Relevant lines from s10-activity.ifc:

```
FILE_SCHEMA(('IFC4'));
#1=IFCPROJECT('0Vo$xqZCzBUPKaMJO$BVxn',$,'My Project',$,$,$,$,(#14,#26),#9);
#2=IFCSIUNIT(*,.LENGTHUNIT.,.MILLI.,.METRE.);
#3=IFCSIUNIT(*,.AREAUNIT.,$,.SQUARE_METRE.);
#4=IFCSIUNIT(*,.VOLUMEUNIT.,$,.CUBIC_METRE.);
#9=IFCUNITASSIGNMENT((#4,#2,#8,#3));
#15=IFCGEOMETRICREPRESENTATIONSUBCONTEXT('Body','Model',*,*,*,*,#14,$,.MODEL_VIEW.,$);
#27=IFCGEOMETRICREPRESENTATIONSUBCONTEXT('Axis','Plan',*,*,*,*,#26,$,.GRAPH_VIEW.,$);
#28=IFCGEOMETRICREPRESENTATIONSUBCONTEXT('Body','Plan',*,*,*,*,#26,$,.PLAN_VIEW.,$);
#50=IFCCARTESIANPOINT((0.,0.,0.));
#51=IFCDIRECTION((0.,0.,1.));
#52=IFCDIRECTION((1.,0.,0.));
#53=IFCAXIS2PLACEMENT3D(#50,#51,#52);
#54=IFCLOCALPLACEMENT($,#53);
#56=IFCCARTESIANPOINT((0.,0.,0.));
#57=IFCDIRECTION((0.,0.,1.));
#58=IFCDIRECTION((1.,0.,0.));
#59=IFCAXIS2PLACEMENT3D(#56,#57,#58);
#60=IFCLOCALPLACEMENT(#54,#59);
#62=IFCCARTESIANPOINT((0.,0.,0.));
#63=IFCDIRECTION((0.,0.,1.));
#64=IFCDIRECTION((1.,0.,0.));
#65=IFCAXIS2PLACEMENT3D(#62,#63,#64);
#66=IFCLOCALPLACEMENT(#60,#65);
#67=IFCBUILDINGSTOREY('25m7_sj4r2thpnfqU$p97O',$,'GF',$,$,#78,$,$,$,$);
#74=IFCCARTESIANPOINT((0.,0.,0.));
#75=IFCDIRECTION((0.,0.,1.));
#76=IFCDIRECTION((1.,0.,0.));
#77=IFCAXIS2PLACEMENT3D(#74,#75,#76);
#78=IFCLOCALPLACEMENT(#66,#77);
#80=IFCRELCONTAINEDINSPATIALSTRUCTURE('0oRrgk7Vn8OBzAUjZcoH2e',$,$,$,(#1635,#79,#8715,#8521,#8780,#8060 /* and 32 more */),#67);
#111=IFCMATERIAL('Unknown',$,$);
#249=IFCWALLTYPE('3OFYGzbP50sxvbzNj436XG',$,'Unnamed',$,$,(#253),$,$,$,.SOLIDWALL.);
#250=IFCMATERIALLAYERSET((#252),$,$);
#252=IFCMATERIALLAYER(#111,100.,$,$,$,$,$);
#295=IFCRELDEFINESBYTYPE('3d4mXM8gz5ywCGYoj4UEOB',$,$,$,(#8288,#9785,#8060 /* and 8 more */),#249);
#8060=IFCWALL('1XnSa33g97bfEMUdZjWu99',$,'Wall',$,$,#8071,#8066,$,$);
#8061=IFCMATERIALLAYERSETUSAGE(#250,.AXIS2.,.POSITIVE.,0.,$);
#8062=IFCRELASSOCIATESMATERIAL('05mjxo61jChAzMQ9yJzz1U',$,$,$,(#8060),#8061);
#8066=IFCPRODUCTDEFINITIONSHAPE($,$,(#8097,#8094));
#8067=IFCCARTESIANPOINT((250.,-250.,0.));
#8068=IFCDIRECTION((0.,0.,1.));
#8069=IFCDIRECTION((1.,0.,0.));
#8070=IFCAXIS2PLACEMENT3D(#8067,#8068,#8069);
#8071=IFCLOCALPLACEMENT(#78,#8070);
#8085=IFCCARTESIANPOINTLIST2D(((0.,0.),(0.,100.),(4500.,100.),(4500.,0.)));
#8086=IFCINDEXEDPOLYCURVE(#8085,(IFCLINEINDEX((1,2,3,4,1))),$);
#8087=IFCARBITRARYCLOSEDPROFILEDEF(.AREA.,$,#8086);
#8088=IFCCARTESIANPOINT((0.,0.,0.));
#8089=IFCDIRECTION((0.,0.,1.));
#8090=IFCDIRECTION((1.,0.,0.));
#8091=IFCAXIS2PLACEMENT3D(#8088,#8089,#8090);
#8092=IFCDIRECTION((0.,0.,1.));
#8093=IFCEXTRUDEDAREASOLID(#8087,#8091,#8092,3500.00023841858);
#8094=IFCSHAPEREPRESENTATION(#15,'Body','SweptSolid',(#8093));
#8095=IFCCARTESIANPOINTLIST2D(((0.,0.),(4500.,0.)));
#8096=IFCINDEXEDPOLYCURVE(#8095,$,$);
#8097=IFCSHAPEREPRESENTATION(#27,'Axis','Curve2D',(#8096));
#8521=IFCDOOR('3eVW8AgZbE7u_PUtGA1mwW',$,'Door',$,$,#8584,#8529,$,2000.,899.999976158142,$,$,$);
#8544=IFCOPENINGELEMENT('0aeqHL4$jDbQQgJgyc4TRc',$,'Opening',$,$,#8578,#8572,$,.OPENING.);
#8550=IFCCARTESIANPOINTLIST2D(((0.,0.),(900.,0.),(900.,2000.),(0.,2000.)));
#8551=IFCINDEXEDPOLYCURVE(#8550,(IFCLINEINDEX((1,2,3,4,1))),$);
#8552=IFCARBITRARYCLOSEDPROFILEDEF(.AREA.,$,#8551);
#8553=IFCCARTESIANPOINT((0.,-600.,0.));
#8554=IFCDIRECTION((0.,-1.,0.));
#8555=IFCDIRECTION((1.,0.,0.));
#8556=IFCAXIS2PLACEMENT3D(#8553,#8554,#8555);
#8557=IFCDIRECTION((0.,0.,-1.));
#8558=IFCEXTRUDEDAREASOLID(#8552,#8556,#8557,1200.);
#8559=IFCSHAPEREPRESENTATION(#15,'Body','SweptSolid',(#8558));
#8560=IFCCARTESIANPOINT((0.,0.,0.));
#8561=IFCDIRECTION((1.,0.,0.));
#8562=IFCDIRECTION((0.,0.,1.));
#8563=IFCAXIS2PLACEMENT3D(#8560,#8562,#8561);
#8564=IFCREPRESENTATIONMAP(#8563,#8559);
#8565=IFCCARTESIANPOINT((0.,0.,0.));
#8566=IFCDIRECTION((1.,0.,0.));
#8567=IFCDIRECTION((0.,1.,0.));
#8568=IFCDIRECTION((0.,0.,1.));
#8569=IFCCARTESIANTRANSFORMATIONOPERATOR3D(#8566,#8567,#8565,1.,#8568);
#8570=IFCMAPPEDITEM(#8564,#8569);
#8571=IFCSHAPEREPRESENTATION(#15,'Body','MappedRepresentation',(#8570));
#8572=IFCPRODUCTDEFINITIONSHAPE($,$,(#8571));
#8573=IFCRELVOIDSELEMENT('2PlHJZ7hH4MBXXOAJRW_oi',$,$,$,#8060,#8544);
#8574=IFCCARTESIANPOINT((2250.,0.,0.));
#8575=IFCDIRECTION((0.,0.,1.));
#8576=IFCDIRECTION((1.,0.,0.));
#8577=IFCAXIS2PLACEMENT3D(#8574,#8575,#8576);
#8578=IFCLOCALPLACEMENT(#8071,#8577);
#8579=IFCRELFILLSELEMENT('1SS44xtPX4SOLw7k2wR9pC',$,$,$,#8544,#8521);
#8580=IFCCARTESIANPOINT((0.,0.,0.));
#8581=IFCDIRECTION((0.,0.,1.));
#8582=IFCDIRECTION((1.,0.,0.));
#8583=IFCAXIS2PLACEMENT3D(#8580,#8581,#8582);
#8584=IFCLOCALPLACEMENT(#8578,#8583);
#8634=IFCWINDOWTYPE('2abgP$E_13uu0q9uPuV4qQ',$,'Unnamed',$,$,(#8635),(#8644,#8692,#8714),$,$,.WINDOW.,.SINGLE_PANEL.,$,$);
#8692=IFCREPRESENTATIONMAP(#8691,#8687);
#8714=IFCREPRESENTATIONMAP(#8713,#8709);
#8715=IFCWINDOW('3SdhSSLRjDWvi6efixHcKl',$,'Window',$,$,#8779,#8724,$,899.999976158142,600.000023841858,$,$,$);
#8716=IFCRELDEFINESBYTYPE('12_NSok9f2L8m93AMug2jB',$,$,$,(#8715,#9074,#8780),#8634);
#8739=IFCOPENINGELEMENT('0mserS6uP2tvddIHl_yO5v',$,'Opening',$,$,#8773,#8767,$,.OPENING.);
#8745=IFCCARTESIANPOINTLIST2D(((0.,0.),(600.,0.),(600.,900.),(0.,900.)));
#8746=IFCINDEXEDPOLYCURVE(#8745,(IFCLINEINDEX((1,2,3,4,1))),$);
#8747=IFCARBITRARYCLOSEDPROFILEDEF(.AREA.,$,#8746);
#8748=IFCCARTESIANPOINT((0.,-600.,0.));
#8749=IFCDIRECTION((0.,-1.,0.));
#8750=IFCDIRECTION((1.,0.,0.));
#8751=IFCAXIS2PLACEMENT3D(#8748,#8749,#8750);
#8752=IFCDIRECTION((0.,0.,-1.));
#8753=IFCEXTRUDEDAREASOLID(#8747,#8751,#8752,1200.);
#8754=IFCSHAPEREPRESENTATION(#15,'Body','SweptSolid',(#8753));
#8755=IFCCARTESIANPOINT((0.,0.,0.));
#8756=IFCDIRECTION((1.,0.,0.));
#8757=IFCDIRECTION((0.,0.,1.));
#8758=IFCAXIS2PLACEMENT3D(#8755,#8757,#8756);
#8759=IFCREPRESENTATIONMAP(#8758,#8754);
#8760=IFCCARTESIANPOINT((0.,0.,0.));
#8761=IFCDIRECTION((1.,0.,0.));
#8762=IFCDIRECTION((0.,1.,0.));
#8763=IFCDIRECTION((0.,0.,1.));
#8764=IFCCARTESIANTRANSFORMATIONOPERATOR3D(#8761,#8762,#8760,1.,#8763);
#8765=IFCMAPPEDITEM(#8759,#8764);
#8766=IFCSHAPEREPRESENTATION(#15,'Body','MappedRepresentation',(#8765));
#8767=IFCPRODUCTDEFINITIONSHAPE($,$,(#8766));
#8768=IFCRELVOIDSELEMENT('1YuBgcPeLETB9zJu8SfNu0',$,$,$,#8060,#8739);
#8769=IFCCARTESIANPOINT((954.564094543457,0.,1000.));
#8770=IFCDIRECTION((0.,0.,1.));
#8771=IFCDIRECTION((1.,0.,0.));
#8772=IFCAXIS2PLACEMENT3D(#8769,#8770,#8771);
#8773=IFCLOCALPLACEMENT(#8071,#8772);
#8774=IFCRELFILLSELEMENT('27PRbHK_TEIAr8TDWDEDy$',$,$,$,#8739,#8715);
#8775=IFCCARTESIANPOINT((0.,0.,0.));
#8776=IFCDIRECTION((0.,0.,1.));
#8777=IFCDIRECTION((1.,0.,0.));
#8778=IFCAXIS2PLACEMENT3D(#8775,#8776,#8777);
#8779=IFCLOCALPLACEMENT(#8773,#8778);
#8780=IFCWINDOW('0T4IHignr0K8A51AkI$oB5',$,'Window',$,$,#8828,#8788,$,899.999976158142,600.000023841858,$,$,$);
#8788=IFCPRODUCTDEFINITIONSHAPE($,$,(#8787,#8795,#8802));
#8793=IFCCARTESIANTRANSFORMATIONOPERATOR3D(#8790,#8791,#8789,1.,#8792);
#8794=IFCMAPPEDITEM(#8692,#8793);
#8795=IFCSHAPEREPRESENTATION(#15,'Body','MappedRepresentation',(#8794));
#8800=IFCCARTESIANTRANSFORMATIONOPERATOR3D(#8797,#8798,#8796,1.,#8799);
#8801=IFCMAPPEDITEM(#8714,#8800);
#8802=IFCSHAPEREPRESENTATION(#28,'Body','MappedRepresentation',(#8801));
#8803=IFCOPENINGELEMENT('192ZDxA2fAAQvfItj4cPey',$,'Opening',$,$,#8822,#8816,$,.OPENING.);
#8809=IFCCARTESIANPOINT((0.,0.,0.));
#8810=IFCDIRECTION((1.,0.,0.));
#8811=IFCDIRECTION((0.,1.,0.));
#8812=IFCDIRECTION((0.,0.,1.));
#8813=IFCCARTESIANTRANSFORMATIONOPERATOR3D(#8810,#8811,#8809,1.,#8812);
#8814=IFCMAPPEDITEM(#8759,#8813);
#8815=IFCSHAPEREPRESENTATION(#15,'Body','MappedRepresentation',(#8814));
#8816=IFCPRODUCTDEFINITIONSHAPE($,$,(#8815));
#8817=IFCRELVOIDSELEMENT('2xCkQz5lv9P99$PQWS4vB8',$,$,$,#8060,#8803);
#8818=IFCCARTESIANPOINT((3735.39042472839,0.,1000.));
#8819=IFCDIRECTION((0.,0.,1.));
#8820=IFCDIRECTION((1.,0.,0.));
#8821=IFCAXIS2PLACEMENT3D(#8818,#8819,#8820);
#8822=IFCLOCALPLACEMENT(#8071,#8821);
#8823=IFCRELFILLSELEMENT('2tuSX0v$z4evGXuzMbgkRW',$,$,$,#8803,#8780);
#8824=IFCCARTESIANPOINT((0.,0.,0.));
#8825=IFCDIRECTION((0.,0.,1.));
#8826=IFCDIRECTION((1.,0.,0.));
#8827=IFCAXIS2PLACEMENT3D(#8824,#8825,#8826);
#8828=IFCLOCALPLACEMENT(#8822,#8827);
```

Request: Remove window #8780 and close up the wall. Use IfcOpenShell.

```python
import ifcopenshell
import ifcopenshell.api.feature
import ifcopenshell.api.root
import ifcopenshell.geom
import ifcopenshell.util.shape

model = ifcopenshell.open("s10-activity.ifc")
settings = ifcopenshell.geom.settings()


def volume(element):
    """Net volume in cubic metres, openings subtracted."""
    shape = ifcopenshell.geom.create_shape(settings, element)
    return ifcopenshell.util.shape.get_volume(shape.geometry)


window = model.by_guid("0T4IHignr0K8A51AkI$oB5")
opening = window.FillsVoids[0].RelatingOpeningElement
wall = opening.VoidsElements[0].RelatingBuildingElement
before = volume(wall)

ifcopenshell.api.root.remove_product(model, product=window)
ifcopenshell.api.feature.remove_feature(model, feature=opening)

after = volume(wall)

print(f"wall volume {before:.3f} -> {after:.3f} m3")

model.write("s10-activity-out.ifc")
```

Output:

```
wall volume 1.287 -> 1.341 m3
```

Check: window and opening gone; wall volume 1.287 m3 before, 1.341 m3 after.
